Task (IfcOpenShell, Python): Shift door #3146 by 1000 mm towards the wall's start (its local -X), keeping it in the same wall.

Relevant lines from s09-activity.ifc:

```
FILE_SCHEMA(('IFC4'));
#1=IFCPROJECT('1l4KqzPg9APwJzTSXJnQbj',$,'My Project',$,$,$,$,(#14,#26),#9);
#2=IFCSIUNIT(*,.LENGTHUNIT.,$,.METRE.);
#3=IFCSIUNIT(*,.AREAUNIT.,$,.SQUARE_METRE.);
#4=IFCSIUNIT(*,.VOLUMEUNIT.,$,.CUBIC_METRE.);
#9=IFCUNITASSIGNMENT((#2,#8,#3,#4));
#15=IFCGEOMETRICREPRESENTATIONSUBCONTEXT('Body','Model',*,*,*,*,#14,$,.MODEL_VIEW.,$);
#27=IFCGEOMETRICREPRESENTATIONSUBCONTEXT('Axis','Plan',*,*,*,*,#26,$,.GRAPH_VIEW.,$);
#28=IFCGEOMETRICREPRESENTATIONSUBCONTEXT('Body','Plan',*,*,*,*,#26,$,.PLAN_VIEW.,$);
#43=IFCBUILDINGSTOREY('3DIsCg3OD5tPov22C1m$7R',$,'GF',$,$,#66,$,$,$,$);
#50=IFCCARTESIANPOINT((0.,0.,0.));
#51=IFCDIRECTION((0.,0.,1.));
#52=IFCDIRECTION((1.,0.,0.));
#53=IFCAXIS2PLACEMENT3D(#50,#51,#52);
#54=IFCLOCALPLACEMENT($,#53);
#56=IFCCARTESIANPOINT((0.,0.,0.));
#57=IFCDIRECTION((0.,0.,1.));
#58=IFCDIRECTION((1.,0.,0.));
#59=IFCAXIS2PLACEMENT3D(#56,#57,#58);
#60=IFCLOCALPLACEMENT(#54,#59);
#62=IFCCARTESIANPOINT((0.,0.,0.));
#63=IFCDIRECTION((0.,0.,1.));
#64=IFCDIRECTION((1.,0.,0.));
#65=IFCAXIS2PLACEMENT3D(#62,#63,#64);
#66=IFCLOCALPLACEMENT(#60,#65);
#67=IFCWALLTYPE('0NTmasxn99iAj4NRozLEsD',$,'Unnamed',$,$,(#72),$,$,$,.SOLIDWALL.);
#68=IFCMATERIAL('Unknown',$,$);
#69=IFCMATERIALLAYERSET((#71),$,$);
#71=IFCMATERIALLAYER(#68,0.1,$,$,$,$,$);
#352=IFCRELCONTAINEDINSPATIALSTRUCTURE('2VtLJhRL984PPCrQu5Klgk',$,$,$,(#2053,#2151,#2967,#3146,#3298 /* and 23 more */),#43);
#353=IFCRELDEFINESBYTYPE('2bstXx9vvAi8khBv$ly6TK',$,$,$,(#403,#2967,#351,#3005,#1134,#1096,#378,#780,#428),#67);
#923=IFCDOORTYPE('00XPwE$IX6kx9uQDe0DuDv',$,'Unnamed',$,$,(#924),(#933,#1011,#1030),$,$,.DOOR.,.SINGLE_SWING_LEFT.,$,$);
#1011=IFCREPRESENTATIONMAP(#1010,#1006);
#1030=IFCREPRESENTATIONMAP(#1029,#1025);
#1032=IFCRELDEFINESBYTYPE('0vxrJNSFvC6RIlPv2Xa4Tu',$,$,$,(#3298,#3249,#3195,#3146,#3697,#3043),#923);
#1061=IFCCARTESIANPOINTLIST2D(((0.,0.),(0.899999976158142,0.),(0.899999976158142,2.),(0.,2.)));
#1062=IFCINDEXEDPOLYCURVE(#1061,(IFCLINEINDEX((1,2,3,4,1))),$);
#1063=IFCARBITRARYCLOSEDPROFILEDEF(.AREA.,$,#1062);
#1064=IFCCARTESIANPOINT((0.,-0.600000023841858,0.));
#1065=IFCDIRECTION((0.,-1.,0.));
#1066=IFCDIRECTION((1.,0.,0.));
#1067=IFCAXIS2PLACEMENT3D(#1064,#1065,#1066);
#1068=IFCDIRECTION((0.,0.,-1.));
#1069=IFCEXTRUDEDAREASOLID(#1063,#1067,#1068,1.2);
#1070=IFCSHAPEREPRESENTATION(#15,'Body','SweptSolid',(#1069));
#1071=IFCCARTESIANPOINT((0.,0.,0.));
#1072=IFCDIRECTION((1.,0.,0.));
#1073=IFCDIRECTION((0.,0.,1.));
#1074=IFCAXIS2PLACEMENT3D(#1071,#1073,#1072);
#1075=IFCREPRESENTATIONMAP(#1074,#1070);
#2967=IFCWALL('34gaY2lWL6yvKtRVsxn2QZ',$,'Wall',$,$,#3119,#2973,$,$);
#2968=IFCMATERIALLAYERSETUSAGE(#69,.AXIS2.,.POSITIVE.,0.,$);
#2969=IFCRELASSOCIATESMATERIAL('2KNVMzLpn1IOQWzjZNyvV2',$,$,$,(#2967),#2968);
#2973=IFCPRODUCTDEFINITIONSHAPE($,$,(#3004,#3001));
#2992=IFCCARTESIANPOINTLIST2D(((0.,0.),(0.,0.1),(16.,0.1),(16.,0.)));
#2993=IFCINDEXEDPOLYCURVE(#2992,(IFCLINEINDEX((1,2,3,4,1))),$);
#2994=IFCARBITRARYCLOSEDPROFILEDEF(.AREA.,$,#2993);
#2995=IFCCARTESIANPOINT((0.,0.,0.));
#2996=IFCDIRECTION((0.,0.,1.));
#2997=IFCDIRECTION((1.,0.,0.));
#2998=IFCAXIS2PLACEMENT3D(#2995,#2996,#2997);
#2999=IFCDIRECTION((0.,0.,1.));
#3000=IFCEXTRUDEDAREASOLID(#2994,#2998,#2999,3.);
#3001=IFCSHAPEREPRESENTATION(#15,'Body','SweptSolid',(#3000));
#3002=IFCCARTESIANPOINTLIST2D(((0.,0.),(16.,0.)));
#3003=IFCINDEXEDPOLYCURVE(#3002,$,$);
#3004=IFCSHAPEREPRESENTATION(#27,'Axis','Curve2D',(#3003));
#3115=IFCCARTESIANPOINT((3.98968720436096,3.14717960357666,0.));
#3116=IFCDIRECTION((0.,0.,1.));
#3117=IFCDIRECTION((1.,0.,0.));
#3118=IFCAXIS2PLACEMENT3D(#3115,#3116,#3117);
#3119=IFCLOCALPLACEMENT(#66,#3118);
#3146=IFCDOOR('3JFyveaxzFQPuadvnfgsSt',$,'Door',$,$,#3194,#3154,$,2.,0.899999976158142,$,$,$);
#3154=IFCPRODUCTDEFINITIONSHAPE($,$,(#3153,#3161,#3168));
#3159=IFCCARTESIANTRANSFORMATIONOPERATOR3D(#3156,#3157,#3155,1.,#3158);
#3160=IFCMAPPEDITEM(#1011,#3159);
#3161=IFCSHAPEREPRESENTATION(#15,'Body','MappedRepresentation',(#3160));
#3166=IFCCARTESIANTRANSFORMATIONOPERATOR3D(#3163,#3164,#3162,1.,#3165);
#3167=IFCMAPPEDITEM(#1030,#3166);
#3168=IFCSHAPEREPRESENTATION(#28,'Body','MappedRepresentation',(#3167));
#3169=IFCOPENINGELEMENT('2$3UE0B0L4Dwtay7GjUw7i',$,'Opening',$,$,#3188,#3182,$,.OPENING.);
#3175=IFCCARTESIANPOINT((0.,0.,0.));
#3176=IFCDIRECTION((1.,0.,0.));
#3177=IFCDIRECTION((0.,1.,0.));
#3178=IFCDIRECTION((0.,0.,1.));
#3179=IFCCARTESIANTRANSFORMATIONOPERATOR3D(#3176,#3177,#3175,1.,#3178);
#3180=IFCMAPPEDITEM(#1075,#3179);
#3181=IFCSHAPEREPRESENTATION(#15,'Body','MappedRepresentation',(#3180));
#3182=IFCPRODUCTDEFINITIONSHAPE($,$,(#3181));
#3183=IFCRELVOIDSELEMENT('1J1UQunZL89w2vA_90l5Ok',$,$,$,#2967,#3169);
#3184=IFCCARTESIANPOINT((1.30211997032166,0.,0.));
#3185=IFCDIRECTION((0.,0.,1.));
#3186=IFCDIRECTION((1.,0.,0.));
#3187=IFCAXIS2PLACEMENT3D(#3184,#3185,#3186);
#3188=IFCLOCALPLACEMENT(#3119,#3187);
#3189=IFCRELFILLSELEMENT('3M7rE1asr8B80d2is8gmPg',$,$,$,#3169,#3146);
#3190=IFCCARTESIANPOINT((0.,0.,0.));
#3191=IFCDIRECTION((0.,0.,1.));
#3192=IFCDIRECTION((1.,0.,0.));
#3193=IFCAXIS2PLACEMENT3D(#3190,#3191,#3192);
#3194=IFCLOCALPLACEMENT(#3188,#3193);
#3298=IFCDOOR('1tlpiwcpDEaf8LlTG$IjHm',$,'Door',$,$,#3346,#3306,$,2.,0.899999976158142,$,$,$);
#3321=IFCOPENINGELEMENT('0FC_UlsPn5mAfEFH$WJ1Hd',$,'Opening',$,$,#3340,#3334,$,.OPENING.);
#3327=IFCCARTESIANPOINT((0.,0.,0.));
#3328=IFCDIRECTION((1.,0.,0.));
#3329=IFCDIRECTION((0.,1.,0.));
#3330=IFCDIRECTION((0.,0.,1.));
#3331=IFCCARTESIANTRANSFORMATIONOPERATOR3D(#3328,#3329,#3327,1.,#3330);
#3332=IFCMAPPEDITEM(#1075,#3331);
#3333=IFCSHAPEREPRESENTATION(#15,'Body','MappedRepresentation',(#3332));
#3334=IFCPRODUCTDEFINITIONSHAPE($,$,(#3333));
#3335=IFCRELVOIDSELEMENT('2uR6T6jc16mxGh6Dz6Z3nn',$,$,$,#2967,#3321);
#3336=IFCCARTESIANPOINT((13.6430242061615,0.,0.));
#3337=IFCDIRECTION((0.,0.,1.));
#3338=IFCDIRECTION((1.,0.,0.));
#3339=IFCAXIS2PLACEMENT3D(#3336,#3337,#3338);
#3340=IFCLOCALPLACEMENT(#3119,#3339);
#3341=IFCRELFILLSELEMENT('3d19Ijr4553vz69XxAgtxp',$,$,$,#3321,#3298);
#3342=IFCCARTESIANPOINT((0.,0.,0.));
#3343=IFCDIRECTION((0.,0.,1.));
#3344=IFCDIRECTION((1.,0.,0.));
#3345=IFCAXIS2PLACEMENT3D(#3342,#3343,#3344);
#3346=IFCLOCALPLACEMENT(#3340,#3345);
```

```python
import ifcopenshell
import ifcopenshell.api.geometry
import ifcopenshell.util.placement
import ifcopenshell.util.unit

model = ifcopenshell.open("s09-activity.ifc")
unit_scale = ifcopenshell.util.unit.calculate_unit_scale(model)

door = model.by_guid("3JFyveaxzFQPuadvnfgsSt")
opening = door.FillsVoids[0].RelatingOpeningElement
wall = opening.VoidsElements[0].RelatingBuildingElement

wall_matrix = ifcopenshell.util.placement.get_local_placement(wall.ObjectPlacement)
shift = wall_matrix[:3, 0] * -1 / unit_scale
before = ifcopenshell.util.placement.get_local_placement(door.ObjectPlacement)[:3, 3].copy()

# The door is placed relative to its opening, so it follows when the opening moves.
matrix = ifcopenshell.util.placement.get_local_placement(opening.ObjectPlacement)
matrix[:3, 3] += shift
ifcopenshell.api.geometry.edit_object_placement(
    model, product=opening, matrix=matrix, is_si=False, should_transform_children=True
)

after = ifcopenshell.util.placement.get_local_placement(door.ObjectPlacement)[:3, 3]
print("door moved by", (after - before).round(3) + 0.0)

model.write("s09-activity_v2.ifc")
```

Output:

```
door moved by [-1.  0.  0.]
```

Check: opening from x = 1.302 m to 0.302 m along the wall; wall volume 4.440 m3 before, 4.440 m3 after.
